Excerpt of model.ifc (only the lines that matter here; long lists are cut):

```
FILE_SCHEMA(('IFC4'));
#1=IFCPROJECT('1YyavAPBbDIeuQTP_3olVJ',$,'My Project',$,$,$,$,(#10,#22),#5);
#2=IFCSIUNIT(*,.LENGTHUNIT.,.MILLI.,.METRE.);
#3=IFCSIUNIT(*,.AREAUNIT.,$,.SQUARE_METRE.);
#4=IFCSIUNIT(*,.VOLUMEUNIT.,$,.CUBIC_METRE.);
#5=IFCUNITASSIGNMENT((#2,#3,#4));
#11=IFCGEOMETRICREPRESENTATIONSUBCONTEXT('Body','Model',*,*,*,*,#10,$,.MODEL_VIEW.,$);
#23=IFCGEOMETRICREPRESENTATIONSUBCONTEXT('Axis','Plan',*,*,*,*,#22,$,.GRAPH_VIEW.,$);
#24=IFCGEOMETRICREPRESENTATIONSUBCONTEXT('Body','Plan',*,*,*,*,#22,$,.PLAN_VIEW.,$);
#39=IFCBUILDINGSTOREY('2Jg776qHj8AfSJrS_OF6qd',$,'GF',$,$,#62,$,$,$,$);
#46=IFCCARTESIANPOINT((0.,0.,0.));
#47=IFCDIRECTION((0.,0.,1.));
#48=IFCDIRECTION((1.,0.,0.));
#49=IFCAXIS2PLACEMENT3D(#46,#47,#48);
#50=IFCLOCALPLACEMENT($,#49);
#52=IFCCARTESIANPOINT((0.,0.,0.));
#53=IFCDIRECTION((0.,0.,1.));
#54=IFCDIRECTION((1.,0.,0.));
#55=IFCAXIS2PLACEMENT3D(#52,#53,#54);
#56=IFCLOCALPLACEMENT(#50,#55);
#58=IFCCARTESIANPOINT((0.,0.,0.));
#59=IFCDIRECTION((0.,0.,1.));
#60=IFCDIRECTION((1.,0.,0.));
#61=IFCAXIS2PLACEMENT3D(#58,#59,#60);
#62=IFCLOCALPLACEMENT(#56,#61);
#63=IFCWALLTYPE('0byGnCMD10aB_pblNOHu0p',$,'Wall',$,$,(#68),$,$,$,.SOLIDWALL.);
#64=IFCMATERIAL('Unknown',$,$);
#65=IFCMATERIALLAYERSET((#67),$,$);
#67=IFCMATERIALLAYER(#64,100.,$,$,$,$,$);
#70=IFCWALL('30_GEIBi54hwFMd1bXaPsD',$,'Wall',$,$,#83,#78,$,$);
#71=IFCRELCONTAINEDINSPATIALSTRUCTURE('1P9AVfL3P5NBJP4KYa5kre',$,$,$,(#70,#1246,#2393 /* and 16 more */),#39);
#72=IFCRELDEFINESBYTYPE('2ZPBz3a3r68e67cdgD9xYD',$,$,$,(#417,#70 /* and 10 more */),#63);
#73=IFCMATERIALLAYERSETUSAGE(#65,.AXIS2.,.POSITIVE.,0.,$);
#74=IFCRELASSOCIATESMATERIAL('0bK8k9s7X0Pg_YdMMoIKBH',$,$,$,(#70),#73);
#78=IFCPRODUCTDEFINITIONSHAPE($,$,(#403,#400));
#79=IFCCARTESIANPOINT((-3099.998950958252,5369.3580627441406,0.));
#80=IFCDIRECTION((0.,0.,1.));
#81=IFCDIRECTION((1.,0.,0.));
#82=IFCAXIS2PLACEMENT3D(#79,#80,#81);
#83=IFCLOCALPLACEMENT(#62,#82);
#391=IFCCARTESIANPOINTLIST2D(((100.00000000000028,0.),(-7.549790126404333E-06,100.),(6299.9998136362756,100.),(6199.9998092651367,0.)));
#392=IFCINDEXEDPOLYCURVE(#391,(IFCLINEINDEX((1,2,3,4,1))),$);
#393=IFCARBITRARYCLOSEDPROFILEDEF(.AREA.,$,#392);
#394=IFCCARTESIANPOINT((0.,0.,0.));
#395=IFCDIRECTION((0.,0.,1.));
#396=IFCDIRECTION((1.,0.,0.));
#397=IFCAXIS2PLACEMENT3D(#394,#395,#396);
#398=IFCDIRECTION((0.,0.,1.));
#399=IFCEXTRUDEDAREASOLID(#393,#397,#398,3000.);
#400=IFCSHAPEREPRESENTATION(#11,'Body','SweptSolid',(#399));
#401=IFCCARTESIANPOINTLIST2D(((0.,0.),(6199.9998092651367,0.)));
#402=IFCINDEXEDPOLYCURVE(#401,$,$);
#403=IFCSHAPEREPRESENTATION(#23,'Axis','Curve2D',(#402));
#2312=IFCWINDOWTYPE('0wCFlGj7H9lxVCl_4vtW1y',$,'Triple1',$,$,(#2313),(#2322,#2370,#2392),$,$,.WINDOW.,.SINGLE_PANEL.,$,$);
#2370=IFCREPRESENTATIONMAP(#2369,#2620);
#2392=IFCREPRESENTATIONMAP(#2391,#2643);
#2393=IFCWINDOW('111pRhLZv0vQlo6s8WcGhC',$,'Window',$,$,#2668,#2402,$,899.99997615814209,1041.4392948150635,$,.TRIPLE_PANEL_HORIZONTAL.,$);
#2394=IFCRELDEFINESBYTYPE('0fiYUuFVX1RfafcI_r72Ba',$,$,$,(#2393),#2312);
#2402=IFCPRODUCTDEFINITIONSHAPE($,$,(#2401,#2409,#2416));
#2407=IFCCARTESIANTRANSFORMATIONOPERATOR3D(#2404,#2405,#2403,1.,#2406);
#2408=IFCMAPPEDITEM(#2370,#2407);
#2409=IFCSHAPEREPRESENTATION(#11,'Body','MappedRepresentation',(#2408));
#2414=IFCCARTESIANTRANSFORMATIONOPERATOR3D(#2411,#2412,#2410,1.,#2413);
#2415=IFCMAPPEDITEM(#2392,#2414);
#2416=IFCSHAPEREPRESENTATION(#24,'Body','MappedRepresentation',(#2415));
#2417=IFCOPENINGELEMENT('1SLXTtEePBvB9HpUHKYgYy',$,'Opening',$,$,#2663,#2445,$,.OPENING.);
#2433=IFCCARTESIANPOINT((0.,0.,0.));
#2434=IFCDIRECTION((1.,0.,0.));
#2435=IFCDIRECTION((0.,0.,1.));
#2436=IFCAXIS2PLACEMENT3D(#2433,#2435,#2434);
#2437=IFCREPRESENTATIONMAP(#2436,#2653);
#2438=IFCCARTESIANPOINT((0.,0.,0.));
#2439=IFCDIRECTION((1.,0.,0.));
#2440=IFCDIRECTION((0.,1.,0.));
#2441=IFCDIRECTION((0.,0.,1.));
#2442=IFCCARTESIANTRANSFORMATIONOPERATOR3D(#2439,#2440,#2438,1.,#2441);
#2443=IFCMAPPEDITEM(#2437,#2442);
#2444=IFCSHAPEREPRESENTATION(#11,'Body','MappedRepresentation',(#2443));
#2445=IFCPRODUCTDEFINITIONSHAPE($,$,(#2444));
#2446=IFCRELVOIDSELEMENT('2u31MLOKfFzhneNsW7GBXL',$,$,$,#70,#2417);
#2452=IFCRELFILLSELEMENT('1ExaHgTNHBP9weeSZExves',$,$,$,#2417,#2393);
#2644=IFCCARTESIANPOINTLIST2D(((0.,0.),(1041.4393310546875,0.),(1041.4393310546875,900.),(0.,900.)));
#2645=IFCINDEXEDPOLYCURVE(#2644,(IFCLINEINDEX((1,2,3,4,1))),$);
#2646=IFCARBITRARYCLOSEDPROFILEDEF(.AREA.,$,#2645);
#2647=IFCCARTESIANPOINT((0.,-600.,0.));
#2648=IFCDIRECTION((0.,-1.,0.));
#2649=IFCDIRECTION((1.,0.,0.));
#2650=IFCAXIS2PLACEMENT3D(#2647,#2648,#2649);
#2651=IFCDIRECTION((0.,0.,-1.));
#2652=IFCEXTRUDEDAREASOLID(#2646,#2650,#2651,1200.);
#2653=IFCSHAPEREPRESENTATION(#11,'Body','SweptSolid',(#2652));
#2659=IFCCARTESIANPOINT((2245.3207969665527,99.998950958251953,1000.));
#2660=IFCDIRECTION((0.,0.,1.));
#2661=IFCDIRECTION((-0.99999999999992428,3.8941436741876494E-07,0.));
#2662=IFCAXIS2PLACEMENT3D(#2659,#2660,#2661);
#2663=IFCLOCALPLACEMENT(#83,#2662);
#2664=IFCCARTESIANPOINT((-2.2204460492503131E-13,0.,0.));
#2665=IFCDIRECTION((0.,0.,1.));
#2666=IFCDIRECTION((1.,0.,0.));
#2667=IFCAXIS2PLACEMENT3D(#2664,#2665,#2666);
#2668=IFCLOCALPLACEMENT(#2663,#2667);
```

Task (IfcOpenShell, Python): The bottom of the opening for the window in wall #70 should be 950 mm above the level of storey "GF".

```python
import numpy as np
import ifcopenshell
import ifcopenshell.api.geometry
import ifcopenshell.geom
import ifcopenshell.util.element
import ifcopenshell.util.placement
import ifcopenshell.util.shape
import ifcopenshell.util.unit

model = ifcopenshell.open("model.ifc")
unit_scale = ifcopenshell.util.unit.calculate_unit_scale(model)

window = model.by_guid("111pRhLZv0vQlo6s8WcGhC")
opening = window.FillsVoids[0].RelatingOpeningElement
storey = ifcopenshell.util.element.get_container(window, ifc_class="IfcBuildingStorey")
level = ifcopenshell.util.placement.get_local_placement(storey.ObjectPlacement)[2, 3]

# The opening's origin need not be at the sill, so measure its lowest point.
shape = ifcopenshell.geom.create_shape(ifcopenshell.geom.settings(), opening)
bottom = ifcopenshell.util.shape.get_shape_bottom_elevation(shape, shape.geometry) / unit_scale
dz = level + 950.0 - bottom

shift = np.array([0.0, 0.0, dz])
# The window is placed relative to its opening, so it follows when the opening moves.
matrix = ifcopenshell.util.placement.get_local_placement(opening.ObjectPlacement)
matrix[:3, 3] += shift
ifcopenshell.api.geometry.edit_object_placement(
    model, product=opening, matrix=matrix, is_si=False, should_transform_children=True
)

print(f"moved by {dz * unit_scale:+.3f} m")

model.write("model_v2.ifc")
```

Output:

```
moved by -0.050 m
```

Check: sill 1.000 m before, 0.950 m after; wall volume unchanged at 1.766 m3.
